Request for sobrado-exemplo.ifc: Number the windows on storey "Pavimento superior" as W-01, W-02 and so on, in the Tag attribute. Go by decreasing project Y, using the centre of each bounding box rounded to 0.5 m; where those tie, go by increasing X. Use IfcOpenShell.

First a look at what the model holds.

```python
import ifcopenshell
import ifcopenshell.util.element
import ifcopenshell.util.placement

model = ifcopenshell.open("sobrado-exemplo.ifc")
print(model.schema)
storey = next(s for s in model.by_type("IfcBuildingStorey") if s.Name == "Pavimento superior")
windows = [e for e in ifcopenshell.util.element.get_decomposition(storey) if e.is_a("IfcWindow")]
for e in sorted(windows, key=lambda e: e.id()):
    origin = ifcopenshell.util.placement.get_local_placement(e.ObjectPlacement)[:3, 3]
    print(e.id(), e.Tag, e.Name, origin.round(2) + 0.0, sep=" | ")
```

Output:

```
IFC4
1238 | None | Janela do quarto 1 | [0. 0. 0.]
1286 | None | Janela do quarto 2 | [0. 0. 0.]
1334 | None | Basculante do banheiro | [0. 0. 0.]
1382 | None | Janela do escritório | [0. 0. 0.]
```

```python
import ifcopenshell
import ifcopenshell.geom
import ifcopenshell.util.element
import ifcopenshell.util.shape

model = ifcopenshell.open("sobrado-exemplo.ifc")
settings = ifcopenshell.geom.settings()
settings.set("use-world-coords", True)


def centre(element):
    shape = ifcopenshell.geom.create_shape(settings, element)
    return ifcopenshell.util.shape.get_bbox_centroid(shape.geometry)


storey = next(s for s in model.by_type("IfcBuildingStorey") if s.Name == "Pavimento superior")
windows = [e for e in ifcopenshell.util.element.get_decomposition(storey) if e.is_a("IfcWindow")]

# Insertion points can sit at a corner or the storey origin, so sort by the geometry (in metres).
centres = {e: centre(e) for e in windows}
windows.sort(key=lambda e: (-round(centres[e][1] / 0.5), centres[e][0]))

for i, e in enumerate(windows, start=1):
    number = f"W-{i:02d}"
    e.Tag = number
    print(e.id(), number)

model.write("sobrado-exemplo-out.ifc")
```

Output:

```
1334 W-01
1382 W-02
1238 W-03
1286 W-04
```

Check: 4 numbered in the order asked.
